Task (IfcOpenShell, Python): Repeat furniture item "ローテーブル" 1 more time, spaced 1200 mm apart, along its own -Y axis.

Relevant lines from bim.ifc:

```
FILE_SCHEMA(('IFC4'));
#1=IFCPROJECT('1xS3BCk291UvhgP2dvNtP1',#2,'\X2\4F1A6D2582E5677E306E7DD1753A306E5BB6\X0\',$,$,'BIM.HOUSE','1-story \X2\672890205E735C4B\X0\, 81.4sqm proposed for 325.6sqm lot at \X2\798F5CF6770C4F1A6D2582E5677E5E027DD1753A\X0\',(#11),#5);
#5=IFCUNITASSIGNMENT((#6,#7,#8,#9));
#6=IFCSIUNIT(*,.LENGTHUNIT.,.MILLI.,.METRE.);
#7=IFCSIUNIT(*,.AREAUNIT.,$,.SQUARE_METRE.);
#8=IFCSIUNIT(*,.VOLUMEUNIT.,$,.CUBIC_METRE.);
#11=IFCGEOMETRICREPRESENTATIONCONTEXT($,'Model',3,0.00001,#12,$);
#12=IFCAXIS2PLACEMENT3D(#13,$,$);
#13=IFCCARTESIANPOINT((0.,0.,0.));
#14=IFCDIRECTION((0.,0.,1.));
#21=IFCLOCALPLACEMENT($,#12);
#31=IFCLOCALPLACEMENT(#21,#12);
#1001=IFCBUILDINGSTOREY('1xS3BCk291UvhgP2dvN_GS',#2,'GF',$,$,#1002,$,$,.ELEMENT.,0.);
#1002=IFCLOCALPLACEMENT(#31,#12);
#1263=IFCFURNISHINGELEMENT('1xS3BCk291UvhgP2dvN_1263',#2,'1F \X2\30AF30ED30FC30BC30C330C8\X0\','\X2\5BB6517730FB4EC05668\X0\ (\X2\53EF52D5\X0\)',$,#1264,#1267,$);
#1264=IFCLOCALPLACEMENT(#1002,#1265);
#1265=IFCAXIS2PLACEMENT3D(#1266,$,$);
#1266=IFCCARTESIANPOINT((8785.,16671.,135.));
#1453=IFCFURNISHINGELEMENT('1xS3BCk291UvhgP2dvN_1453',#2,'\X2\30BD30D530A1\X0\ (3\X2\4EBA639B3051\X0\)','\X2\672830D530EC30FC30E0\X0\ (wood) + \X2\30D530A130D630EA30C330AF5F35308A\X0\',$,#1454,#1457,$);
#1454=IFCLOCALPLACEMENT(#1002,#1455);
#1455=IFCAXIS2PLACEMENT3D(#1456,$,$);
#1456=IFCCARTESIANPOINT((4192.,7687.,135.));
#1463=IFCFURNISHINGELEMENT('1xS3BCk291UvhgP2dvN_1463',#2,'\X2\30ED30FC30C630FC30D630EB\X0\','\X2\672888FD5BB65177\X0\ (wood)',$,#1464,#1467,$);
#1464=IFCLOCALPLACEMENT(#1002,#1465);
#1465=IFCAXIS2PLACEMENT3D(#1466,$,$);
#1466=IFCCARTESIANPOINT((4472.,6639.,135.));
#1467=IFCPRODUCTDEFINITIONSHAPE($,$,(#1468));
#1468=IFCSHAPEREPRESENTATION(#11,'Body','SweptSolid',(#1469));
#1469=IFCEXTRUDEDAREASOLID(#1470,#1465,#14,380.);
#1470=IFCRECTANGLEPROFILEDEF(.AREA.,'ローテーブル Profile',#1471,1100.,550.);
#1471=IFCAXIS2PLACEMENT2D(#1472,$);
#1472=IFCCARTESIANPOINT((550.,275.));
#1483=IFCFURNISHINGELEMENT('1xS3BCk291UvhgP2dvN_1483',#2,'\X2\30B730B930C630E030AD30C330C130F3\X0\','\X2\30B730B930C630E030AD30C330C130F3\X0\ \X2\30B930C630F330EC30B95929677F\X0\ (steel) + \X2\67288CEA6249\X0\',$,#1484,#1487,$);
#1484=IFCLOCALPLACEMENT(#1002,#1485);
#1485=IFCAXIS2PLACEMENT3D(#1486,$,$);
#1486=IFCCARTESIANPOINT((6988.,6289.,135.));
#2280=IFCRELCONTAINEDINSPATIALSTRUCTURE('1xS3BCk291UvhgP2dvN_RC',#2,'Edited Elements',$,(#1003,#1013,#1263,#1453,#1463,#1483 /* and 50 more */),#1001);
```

```python
import ifcopenshell
import ifcopenshell.api.geometry
import ifcopenshell.api.root
import ifcopenshell.util.element
import ifcopenshell.util.placement
import ifcopenshell.util.unit

model = ifcopenshell.open("bim.ifc")
unit_scale = ifcopenshell.util.unit.calculate_unit_scale(model)


def reuse_history(source, copy):
    """copy_class also copies each property set's owner history, people and application; keep the originals."""
    for rel in copy.IsDefinedBy:
        if rel.is_a("IfcRelDefinesByProperties") and (history := rel.RelatingPropertyDefinition.OwnerHistory):
            rel.RelatingPropertyDefinition.OwnerHistory = source.OwnerHistory
            ifcopenshell.util.element.remove_deep2(model, history)


source = model.by_guid("1xS3BCk291UvhgP2dvN_1463")
base = ifcopenshell.util.placement.get_local_placement(source.ObjectPlacement)
step = -base[:3, 1] * 1.2 / unit_scale

for i in range(1, 2):
    copy = ifcopenshell.api.root.copy_class(model, product=source)
    copy.Representation = ifcopenshell.util.element.copy_deep(
        model, source.Representation, exclude=["IfcGeometricRepresentationContext", "IfcRepresentationMap"]
    )
    reuse_history(source, copy)
    matrix = base.copy()
    matrix[:3, 3] += i * step
    print("added at", matrix[:3, 3].round(3) + 0.0)
    ifcopenshell.api.geometry.edit_object_placement(model, product=copy, matrix=matrix, is_si=False)

model.write("bim_v2.ifc")
```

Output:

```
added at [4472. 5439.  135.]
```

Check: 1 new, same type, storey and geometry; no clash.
